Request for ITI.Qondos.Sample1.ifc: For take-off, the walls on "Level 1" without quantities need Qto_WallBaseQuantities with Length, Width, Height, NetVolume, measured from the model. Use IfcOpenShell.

First a look at what the model holds.

```python
import ifcopenshell
import ifcopenshell.util.element
import ifcopenshell.util.unit

model = ifcopenshell.open("ITI.Qondos.Sample1.ifc")
print(model.schema)
for unit_type in ("LENGTHUNIT", "AREAUNIT", "VOLUMEUNIT"):
    print(unit_type, ifcopenshell.util.unit.calculate_unit_scale(model, unit_type))
storey = next(s for s in model.by_type("IfcBuildingStorey") if s.Name == "Level 1")
walls = [e for e in ifcopenshell.util.element.get_decomposition(storey) if e.is_a("IfcWall")]
for e in sorted(walls, key=lambda e: e.id()):
    print(e.id(), e.is_a(), e.Name, list(ifcopenshell.util.element.get_psets(e, qtos_only=True)), sep=" | ")
```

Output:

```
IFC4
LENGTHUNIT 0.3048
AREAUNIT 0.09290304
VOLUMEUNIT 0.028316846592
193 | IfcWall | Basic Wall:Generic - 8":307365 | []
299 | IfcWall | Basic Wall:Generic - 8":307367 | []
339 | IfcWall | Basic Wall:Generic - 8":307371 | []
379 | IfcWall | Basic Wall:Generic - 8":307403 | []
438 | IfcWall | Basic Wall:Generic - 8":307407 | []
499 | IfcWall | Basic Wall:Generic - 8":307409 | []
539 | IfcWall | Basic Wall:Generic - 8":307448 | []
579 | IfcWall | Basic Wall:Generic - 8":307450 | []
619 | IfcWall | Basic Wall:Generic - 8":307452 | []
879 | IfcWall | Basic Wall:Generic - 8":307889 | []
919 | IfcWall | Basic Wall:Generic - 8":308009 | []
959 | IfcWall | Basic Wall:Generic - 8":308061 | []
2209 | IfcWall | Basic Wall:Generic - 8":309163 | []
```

```python
import ifcopenshell
import ifcopenshell.api.pset
import ifcopenshell.geom
import ifcopenshell.util.element
import ifcopenshell.util.shape
import ifcopenshell.util.unit

model = ifcopenshell.open("ITI.Qondos.Sample1.ifc")
unit_scale = ifcopenshell.util.unit.calculate_unit_scale(model)
volume_scale = ifcopenshell.util.unit.calculate_unit_scale(model, "VOLUMEUNIT")
settings = ifcopenshell.geom.settings()

storey = next(s for s in model.by_type("IfcBuildingStorey") if s.Name == "Level 1")
walls = [e for e in ifcopenshell.util.element.get_decomposition(storey) if e.is_a("IfcWall")]

for e in sorted(walls, key=lambda e: e.id()):
    if ifcopenshell.util.element.get_psets(e, qtos_only=True, should_inherit=False):
        continue
    # Geometry comes back in metres, in the element's own axes.
    shape = ifcopenshell.geom.create_shape(settings, e)
    values = {
        "Length": ifcopenshell.util.shape.get_x(shape.geometry) / unit_scale,
        "Width": ifcopenshell.util.shape.get_y(shape.geometry) / unit_scale,
        "Height": ifcopenshell.util.shape.get_z(shape.geometry) / unit_scale,
        "NetVolume": ifcopenshell.util.shape.get_volume(shape.geometry) / volume_scale,
    }
    qto = ifcopenshell.api.pset.add_qto(model, product=e, name="Qto_WallBaseQuantities")
    ifcopenshell.api.pset.edit_qto(model, qto=qto, properties=values)
    print(e.id(), {k: round(v, 3) for k, v in values.items()})

model.write("ITI.Qondos.Sample1_v2.ifc")
```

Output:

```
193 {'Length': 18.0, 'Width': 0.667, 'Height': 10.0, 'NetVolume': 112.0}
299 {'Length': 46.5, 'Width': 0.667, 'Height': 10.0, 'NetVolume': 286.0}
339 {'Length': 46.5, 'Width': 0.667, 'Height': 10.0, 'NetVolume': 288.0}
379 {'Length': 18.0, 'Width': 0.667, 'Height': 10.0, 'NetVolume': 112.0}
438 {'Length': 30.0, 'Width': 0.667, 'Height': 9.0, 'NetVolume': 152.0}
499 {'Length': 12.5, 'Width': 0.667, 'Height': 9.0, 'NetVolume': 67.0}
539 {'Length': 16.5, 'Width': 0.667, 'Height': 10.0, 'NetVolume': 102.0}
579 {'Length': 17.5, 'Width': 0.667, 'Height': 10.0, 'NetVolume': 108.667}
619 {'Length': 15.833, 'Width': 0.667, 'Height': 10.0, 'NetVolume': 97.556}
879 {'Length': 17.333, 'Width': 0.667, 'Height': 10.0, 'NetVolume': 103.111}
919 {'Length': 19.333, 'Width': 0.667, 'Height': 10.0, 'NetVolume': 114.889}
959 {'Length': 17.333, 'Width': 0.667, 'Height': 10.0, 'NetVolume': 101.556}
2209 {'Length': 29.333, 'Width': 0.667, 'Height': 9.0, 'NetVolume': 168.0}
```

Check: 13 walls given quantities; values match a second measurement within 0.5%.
